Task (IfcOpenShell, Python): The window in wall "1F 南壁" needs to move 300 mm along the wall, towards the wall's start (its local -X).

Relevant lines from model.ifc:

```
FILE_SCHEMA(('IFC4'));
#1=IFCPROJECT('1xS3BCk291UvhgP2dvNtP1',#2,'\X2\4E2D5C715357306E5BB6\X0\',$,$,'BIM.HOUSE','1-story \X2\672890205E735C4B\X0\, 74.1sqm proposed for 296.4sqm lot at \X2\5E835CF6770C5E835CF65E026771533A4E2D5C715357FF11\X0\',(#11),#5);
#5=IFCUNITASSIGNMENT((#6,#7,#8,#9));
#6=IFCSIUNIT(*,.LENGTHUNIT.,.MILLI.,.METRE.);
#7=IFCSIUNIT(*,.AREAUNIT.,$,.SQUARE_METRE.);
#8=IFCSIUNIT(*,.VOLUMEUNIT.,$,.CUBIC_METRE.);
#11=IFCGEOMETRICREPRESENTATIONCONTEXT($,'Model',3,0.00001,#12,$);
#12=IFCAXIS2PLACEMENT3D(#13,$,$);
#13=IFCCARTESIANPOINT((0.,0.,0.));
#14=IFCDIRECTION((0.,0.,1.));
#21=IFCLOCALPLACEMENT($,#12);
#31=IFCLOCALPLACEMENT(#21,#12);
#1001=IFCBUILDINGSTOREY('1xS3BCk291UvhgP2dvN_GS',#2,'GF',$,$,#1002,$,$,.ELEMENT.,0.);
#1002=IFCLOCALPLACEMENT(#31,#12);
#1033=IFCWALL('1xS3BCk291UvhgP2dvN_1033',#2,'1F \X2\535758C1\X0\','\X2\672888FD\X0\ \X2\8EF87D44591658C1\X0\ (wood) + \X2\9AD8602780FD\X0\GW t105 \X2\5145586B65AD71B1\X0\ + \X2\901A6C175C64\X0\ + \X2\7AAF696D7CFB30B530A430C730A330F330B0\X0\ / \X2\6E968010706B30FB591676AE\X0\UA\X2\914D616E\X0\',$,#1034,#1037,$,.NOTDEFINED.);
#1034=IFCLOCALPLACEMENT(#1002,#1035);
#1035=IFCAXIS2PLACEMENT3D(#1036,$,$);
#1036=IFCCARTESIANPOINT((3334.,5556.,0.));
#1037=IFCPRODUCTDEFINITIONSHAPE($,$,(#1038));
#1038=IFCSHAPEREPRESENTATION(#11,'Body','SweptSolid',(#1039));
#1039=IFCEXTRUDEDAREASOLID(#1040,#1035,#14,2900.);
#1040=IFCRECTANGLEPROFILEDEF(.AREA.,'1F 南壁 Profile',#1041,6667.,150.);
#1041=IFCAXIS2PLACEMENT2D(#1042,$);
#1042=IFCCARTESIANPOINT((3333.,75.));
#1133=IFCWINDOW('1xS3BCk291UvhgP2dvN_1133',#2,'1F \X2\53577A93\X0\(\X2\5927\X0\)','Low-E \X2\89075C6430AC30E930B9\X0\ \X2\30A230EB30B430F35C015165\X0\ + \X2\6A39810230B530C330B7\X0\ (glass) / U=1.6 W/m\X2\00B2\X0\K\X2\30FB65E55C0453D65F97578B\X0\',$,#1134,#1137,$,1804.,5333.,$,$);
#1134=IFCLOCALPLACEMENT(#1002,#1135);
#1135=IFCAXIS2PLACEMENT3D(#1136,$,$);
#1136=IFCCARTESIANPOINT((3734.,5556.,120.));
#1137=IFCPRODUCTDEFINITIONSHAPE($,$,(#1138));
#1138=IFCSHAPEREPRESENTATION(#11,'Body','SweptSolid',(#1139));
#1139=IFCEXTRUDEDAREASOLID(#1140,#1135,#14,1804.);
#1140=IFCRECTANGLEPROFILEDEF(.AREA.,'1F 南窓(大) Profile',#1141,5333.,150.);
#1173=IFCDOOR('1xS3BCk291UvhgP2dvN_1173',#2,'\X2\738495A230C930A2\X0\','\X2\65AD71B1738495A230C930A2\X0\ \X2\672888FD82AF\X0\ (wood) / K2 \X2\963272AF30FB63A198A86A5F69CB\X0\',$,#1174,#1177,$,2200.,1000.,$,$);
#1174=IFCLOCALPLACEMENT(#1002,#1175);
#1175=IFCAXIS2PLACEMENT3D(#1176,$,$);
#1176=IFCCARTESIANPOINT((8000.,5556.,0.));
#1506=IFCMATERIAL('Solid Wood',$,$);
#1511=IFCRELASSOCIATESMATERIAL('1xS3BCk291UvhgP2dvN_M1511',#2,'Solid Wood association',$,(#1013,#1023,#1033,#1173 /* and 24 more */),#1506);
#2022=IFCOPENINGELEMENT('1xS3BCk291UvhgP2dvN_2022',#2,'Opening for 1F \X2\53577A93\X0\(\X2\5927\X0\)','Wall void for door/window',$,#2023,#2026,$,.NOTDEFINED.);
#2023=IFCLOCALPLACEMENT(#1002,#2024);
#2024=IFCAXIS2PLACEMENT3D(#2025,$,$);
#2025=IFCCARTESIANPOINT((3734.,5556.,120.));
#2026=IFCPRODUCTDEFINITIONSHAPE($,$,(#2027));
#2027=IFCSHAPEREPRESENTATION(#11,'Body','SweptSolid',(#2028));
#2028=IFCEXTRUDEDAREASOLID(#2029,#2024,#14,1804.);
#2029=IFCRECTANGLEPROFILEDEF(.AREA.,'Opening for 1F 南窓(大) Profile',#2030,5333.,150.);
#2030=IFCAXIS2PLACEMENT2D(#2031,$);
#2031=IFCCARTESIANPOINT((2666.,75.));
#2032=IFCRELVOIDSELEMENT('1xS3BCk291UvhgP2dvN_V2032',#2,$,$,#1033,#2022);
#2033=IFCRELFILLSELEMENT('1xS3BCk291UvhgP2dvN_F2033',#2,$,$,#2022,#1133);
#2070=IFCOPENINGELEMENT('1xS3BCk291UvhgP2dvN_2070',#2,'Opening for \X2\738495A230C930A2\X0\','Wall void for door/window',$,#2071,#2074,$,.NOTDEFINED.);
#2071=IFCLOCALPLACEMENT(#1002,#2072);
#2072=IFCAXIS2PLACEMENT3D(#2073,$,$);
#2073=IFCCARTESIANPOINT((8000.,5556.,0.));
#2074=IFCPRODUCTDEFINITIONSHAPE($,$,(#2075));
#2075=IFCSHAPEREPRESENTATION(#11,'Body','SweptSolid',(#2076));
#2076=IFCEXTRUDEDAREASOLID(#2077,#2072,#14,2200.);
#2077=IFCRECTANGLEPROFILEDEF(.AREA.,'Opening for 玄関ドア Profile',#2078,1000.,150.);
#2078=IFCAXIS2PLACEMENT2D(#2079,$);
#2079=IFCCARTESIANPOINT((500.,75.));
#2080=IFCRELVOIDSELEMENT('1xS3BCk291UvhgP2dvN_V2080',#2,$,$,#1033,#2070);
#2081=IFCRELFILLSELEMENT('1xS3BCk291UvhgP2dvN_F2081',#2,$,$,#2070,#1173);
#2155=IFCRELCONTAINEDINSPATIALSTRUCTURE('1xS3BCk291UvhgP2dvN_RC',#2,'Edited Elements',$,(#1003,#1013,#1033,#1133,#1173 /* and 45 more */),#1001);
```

```python
import ifcopenshell
import ifcopenshell.api.geometry
import ifcopenshell.util.placement
import ifcopenshell.util.unit

model = ifcopenshell.open("model.ifc")
unit_scale = ifcopenshell.util.unit.calculate_unit_scale(model)

window = model.by_guid("1xS3BCk291UvhgP2dvN_1133")
opening = window.FillsVoids[0].RelatingOpeningElement
wall = opening.VoidsElements[0].RelatingBuildingElement

wall_matrix = ifcopenshell.util.placement.get_local_placement(wall.ObjectPlacement)
shift = wall_matrix[:3, 0] * -0.3 / unit_scale
before = ifcopenshell.util.placement.get_local_placement(window.ObjectPlacement)[:3, 3].copy()

# The window is not placed relative to its opening, so move both.
for product in (opening, window):
    matrix = ifcopenshell.util.placement.get_local_placement(product.ObjectPlacement)
    matrix[:3, 3] += shift
    ifcopenshell.api.geometry.edit_object_placement(model, product=product, matrix=matrix, is_si=False)

after = ifcopenshell.util.placement.get_local_placement(window.ObjectPlacement)[:3, 3]
print("window moved by", (after - before).round(3) + 0.0)

model.write("model_v2.ifc")
```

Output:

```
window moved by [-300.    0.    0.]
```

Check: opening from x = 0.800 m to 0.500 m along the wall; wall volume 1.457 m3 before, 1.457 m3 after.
